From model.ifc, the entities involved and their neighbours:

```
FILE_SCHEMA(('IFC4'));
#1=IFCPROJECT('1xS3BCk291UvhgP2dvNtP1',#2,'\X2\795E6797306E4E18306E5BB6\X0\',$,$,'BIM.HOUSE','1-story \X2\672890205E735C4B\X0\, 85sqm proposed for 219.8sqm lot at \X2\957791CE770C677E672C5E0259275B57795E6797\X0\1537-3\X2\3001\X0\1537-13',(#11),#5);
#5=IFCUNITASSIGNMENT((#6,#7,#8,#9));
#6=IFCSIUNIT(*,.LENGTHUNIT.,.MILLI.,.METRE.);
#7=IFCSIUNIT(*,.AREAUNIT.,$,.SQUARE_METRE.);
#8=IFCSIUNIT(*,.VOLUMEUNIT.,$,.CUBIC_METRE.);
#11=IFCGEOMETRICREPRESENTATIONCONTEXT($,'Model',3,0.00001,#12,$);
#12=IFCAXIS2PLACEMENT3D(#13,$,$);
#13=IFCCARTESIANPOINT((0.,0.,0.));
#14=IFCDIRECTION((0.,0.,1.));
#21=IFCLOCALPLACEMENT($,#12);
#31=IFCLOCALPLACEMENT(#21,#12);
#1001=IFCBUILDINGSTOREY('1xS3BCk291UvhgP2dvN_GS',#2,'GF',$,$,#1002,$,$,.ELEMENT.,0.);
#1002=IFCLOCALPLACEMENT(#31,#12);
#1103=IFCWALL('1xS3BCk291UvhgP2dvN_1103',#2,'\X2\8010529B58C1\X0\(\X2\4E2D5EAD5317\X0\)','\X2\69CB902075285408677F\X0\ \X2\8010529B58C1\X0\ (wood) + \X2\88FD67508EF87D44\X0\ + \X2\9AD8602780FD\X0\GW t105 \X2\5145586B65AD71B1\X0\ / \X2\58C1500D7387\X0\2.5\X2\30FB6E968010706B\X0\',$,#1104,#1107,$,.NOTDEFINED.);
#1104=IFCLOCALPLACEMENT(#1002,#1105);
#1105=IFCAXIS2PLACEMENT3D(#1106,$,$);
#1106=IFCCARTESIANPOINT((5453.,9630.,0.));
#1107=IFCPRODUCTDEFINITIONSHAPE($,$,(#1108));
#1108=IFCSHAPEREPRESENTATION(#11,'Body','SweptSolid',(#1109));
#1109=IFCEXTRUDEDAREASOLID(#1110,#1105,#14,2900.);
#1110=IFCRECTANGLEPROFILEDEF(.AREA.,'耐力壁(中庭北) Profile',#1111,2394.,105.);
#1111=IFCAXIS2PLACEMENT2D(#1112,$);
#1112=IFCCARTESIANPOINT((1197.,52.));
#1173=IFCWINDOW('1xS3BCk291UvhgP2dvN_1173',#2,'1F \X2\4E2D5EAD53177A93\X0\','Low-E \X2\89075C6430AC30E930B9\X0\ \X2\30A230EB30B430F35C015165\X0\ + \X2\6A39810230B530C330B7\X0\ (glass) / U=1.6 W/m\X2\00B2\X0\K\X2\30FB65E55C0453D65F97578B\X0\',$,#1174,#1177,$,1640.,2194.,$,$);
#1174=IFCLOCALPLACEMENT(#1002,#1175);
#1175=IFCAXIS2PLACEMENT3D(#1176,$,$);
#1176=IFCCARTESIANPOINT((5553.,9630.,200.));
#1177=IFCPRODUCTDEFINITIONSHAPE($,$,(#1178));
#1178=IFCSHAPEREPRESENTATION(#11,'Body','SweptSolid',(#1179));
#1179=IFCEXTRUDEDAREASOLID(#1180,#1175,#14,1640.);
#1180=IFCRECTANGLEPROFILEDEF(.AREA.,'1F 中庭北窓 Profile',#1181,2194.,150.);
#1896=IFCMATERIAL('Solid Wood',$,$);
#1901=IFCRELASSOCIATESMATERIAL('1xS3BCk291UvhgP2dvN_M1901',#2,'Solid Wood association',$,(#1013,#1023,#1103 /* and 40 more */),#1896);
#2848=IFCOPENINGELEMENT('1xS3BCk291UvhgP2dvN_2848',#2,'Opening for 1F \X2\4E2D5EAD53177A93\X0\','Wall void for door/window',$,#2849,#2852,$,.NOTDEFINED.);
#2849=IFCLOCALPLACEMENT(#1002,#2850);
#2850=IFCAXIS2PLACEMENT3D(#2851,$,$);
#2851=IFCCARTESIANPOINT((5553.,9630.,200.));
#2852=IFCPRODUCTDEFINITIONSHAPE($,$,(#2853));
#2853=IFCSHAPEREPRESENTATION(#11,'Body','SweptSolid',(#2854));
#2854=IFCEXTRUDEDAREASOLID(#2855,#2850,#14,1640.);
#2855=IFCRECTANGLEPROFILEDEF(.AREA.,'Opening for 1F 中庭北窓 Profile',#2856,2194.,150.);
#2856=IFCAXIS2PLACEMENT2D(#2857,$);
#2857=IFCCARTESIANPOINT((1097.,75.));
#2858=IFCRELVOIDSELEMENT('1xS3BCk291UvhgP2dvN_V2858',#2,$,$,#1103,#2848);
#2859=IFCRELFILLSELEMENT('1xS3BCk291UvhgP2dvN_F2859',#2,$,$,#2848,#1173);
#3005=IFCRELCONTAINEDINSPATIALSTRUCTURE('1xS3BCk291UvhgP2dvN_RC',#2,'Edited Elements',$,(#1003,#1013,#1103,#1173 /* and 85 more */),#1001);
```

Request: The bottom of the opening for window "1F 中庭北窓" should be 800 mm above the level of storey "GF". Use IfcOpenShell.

```python
import numpy as np
import ifcopenshell
import ifcopenshell.api.geometry
import ifcopenshell.geom
import ifcopenshell.util.element
import ifcopenshell.util.placement
import ifcopenshell.util.shape
import ifcopenshell.util.unit

model = ifcopenshell.open("model.ifc")
unit_scale = ifcopenshell.util.unit.calculate_unit_scale(model)

window = model.by_guid("1xS3BCk291UvhgP2dvN_1173")
opening = window.FillsVoids[0].RelatingOpeningElement
storey = ifcopenshell.util.element.get_container(window, ifc_class="IfcBuildingStorey")
level = ifcopenshell.util.placement.get_local_placement(storey.ObjectPlacement)[2, 3]

# The opening's origin need not be at the sill, so measure its lowest point.
shape = ifcopenshell.geom.create_shape(ifcopenshell.geom.settings(), opening)
bottom = ifcopenshell.util.shape.get_shape_bottom_elevation(shape, shape.geometry) / unit_scale
dz = level + 0.8 / unit_scale - bottom

shift = np.array([0.0, 0.0, dz])
# The window is not placed relative to its opening, so move both.
for product in (opening, window):
    matrix = ifcopenshell.util.placement.get_local_placement(product.ObjectPlacement)
    matrix[:3, 3] += shift
    ifcopenshell.api.geometry.edit_object_placement(model, product=product, matrix=matrix, is_si=False)

print(f"moved by {dz * unit_scale:+.3f} m")

model.write("model_updated.ifc")
```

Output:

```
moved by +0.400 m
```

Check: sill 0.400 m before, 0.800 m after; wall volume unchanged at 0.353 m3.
